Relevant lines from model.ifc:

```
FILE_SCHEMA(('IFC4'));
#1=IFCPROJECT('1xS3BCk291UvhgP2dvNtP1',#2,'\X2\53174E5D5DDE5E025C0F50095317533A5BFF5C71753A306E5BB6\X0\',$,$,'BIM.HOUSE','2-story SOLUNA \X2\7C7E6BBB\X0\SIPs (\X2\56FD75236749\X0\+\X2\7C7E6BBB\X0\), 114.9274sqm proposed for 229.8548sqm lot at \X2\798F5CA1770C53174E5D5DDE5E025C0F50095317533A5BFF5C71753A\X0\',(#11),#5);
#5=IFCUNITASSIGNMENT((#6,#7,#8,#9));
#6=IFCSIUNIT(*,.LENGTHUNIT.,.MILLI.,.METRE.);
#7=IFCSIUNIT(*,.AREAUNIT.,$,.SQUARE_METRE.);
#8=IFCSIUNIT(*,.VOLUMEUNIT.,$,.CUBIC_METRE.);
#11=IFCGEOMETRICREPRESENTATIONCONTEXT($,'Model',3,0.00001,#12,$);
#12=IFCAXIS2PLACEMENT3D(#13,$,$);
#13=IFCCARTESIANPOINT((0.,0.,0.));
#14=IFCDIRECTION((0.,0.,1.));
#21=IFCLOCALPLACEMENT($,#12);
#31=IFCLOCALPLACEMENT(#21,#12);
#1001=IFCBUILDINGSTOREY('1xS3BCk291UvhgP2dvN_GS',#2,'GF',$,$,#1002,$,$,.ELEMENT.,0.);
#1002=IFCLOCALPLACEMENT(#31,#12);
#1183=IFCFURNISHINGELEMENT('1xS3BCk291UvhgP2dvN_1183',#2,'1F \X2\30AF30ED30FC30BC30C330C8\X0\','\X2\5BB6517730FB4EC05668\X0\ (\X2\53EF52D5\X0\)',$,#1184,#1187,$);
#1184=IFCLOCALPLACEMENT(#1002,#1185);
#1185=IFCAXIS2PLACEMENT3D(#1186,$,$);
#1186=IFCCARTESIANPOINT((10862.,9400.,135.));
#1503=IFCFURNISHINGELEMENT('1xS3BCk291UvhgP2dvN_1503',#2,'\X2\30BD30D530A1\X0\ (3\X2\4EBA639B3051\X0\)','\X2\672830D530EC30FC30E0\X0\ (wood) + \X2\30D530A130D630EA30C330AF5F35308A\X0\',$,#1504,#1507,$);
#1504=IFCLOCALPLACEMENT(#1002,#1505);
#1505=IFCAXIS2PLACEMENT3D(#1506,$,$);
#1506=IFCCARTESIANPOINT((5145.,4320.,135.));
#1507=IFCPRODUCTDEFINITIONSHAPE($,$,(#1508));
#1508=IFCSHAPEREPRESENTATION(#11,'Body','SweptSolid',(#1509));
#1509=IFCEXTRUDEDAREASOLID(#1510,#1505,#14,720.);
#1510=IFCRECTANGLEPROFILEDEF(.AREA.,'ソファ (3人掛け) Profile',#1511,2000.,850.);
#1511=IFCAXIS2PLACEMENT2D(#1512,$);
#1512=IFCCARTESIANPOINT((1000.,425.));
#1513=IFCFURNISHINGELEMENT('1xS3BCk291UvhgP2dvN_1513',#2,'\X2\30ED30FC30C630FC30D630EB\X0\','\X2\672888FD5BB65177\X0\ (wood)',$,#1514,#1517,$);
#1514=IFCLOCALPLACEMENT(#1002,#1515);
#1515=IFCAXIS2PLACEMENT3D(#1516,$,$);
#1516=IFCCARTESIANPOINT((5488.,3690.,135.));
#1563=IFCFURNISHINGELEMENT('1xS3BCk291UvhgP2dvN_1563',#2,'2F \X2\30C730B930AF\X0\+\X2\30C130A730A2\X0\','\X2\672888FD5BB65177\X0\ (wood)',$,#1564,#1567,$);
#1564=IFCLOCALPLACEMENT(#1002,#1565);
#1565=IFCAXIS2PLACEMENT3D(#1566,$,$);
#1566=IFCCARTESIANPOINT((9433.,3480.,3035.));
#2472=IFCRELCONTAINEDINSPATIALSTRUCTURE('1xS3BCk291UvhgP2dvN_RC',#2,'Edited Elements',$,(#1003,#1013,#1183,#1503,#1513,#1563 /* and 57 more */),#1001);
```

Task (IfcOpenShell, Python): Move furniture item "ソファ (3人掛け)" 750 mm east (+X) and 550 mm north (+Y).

```python
import ifcopenshell
import ifcopenshell.api.geometry
import ifcopenshell.util.placement

model = ifcopenshell.open("model.ifc")

item = model.by_guid("1xS3BCk291UvhgP2dvN_1503")
matrix = ifcopenshell.util.placement.get_local_placement(item.ObjectPlacement)
matrix[0, 3] += 750.0
matrix[1, 3] += 550.0
ifcopenshell.api.geometry.edit_object_placement(model, product=item, matrix=matrix, is_si=False)

print(ifcopenshell.util.placement.get_local_placement(item.ObjectPlacement).round(3) + 0.0)

model.write("model_updated.ifc")
```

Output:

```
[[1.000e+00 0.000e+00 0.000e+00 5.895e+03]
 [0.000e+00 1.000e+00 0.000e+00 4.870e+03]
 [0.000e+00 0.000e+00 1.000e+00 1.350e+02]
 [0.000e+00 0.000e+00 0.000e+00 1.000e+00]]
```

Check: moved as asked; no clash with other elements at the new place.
